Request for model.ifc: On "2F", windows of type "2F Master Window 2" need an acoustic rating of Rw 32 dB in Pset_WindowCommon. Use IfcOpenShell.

First a look at what the model holds.

```python
import ifcopenshell
import ifcopenshell.util.element

model = ifcopenshell.open("model.ifc")
print(model.schema)
storey = next(s for s in model.by_type("IfcBuildingStorey") if s.Name == "2F")
windows = [e for e in ifcopenshell.util.element.get_decomposition(storey) if e.is_a("IfcWindow")]
seen = {}
for e in windows:
    element_type = ifcopenshell.util.element.get_type(e)
    key = (element_type.Name if element_type != e and element_type else None, ifcopenshell.util.element.get_pset(e, "Pset_WindowCommon", "AcousticRating"))
    seen[key] = seen.get(key, 0) + 1
for (name, value), count in sorted(seen.items(), key=str):
    print(count, "x", name, "|", value)
```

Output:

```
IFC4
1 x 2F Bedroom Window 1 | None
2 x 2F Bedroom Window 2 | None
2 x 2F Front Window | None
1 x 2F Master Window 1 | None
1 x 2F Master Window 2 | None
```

```python
import ifcopenshell
import ifcopenshell.api.pset
import ifcopenshell.util.element

model = ifcopenshell.open("model.ifc")

storey = next(s for s in model.by_type("IfcBuildingStorey") if s.Name == "2F")
windows = [e for e in ifcopenshell.util.element.get_decomposition(storey) if e.is_a("IfcWindow")]

count = 0
for e in windows:
    element_type = ifcopenshell.util.element.get_type(e)
    if element_type in (None, e) or element_type.Name != "2F Master Window 2":
        continue
    # add_pset returns the element's existing set when there is one.
    pset = ifcopenshell.api.pset.add_pset(model, product=e, name="Pset_WindowCommon")
    ifcopenshell.api.pset.edit_pset(model, pset=pset, properties={"AcousticRating": "Rw 32 dB"})
    count += 1

print(count, "windows updated")

model.write("model_v2.ifc")
```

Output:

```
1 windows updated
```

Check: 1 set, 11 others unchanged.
